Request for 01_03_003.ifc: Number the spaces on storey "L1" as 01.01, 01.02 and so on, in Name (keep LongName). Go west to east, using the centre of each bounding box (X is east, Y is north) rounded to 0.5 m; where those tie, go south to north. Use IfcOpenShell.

First a look at what the model holds.

```python
import ifcopenshell
import ifcopenshell.util.element
import ifcopenshell.util.placement

model = ifcopenshell.open("01_03_003.ifc")
print(model.schema)
storey = next(s for s in model.by_type("IfcBuildingStorey") if s.Name == "L1")
spaces = [e for e in ifcopenshell.util.element.get_decomposition(storey) if e.is_a("IfcSpace")]
for e in sorted(spaces, key=lambda e: e.id()):
    origin = ifcopenshell.util.placement.get_local_placement(e.ObjectPlacement)[:3, 3]
    print(e.id(), e.Name, e.LongName, origin.round(2) + 0.0, sep=" | ")
```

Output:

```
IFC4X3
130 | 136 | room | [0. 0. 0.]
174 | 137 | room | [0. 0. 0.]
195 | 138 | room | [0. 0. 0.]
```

```python
import ifcopenshell
import ifcopenshell.geom
import ifcopenshell.util.element
import ifcopenshell.util.shape

model = ifcopenshell.open("01_03_003.ifc")
settings = ifcopenshell.geom.settings()
settings.set("use-world-coords", True)


def centre(element):
    shape = ifcopenshell.geom.create_shape(settings, element)
    return ifcopenshell.util.shape.get_bbox_centroid(shape.geometry)


storey = next(s for s in model.by_type("IfcBuildingStorey") if s.Name == "L1")
spaces = [e for e in ifcopenshell.util.element.get_decomposition(storey) if e.is_a("IfcSpace")]

# Insertion points can sit at a corner or the storey origin, so sort by the geometry (in metres).
centres = {e: centre(e) for e in spaces}
spaces.sort(key=lambda e: (round(centres[e][0] / 0.5), centres[e][1]))

for i, e in enumerate(spaces, start=1):
    number = f"01.{i:02d}"
    e.Name = number
    print(e.id(), number)

model.write("01_03_003_updated.ifc")
```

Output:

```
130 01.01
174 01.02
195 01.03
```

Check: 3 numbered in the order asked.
